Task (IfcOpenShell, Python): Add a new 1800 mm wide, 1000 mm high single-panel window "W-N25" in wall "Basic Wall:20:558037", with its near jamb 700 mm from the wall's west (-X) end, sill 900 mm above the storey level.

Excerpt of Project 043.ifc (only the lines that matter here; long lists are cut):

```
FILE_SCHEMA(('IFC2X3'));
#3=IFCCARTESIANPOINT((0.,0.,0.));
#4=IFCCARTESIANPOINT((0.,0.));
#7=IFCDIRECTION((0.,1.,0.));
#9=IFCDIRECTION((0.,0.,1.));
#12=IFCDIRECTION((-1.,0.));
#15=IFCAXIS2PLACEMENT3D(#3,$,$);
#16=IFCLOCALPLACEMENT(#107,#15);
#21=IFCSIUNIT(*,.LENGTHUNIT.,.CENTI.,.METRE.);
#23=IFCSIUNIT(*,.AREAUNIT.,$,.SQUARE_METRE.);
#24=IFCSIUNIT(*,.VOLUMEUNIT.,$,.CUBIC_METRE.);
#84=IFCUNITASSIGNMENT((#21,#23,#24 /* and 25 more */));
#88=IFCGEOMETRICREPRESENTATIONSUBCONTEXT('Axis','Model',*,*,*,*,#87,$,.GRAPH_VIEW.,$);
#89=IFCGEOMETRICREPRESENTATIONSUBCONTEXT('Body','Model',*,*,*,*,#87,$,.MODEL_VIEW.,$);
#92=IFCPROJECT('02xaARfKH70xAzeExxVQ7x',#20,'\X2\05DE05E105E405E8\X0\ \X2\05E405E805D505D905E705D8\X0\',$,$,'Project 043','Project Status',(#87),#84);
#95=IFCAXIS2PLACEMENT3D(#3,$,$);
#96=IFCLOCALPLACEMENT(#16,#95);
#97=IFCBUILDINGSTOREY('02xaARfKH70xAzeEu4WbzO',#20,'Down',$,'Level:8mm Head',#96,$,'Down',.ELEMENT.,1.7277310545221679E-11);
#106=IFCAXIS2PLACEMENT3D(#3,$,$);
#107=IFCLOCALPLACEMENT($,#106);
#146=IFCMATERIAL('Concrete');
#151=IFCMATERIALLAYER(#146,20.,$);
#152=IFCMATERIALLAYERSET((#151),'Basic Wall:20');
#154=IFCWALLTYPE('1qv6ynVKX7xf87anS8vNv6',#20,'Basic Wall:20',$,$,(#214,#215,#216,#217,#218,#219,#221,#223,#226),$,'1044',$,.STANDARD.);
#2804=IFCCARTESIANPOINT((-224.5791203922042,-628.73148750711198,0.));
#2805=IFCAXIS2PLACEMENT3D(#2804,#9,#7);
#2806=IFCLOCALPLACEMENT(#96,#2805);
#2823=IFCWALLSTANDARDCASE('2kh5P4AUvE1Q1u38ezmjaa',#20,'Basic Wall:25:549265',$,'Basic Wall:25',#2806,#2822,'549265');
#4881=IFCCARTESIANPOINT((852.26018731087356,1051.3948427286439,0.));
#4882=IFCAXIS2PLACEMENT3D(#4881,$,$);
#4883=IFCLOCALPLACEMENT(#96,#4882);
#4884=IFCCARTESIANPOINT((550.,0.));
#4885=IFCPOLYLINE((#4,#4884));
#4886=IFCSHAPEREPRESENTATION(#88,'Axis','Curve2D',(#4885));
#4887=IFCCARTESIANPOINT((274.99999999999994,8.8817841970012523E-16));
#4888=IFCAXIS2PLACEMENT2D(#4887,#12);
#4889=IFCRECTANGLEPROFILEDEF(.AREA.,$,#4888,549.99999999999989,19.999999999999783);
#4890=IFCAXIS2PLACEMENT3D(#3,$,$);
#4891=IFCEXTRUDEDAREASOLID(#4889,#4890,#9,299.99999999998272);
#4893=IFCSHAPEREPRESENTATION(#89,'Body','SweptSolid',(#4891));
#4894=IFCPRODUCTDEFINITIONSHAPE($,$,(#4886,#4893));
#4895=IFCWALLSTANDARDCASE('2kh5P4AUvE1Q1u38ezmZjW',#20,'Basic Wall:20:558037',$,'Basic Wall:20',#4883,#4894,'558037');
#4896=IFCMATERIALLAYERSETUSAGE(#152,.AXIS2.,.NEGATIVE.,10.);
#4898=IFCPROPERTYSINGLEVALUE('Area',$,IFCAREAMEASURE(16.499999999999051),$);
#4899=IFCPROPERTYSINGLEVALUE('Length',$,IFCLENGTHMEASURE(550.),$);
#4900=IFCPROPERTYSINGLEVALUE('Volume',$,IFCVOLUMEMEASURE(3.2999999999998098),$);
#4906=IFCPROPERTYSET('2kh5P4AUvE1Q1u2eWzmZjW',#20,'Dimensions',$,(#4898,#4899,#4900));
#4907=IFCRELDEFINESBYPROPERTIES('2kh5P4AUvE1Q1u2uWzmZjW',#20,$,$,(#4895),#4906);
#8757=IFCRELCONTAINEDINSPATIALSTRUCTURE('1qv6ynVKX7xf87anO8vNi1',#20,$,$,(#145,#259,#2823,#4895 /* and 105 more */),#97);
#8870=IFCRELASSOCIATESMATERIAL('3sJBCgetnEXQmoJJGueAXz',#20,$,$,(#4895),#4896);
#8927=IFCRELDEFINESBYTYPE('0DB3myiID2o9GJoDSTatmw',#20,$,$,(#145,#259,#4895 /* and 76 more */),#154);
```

```python
import numpy as np
import ifcopenshell
import ifcopenshell.api.feature
import ifcopenshell.api.geometry
import ifcopenshell.api.pset
import ifcopenshell.api.root
import ifcopenshell.api.spatial
import ifcopenshell.api.type
import ifcopenshell.geom
import ifcopenshell.util.element
import ifcopenshell.util.placement
import ifcopenshell.util.representation
import ifcopenshell.util.shape
import ifcopenshell.util.unit

model = ifcopenshell.open("Project 043.ifc")
unit_scale = ifcopenshell.util.unit.calculate_unit_scale(model)
area_scale = ifcopenshell.util.unit.calculate_unit_scale(model, "AREAUNIT")
volume_scale = ifcopenshell.util.unit.calculate_unit_scale(model, "VOLUMEUNIT")
settings = ifcopenshell.geom.settings()


def volume(element):
    """Net volume in cubic metres, openings subtracted."""
    shape = ifcopenshell.geom.create_shape(settings, element)
    return ifcopenshell.util.shape.get_volume(shape.geometry)


wall = model.by_id(4895)
storey = ifcopenshell.util.element.get_container(wall, ifc_class="IfcBuildingStorey")
context = ifcopenshell.util.representation.get_context(model, "Model", "Body", "MODEL_VIEW")
before = volume(wall)

width, height, from_end, sill = 1.8, 1, 0.7, 0.9  # metres

# The wall runs along its own X axis, and the end named is its -X end.
wall_shape = ifcopenshell.geom.create_shape(settings, wall)
x, y, z = ifcopenshell.util.shape.get_vertices(wall_shape.geometry).T
start = x.min() + from_end
face, thickness = float(y.min()), float(y.max() - y.min())
wall_matrix = ifcopenshell.util.placement.get_local_placement(wall.ObjectPlacement)
level = ifcopenshell.util.placement.get_local_placement(storey.ObjectPlacement)[2, 3]


def in_wall(x, y):
    """Placement at x, y metres in the wall's axes, at sill height."""
    matrix = wall_matrix.copy()
    matrix[:, 3] = wall_matrix @ np.array([x / unit_scale, y / unit_scale, 0.0, 1.0])
    matrix[2, 3] = level + sill / unit_scale
    return matrix


# Opening: a box that overshoots both wall faces by 50 mm.
opening = ifcopenshell.api.root.create_entity(model, ifc_class="IfcOpeningElement")
box = ifcopenshell.api.geometry.add_wall_representation(
    model, context=context, length=width, height=height, thickness=thickness + 0.1
)
ifcopenshell.api.geometry.assign_representation(model, product=opening, representation=box)
ifcopenshell.api.geometry.edit_object_placement(model, product=opening, matrix=in_wall(start, face - 0.05), is_si=False)
ifcopenshell.api.feature.add_feature(model, feature=opening, element=wall)

window = ifcopenshell.api.root.create_entity(model, ifc_class="IfcWindow", name="W-N25")
window.OverallWidth, window.OverallHeight = width / unit_scale, height / unit_scale
body = ifcopenshell.api.geometry.add_window_representation(
    model,
    context=context,
    overall_width=window.OverallWidth,
    overall_height=window.OverallHeight,
    partition_type="SINGLE_PANEL",
)
ifcopenshell.api.geometry.assign_representation(model, product=window, representation=body)
ifcopenshell.api.spatial.assign_container(model, products=[window], relating_structure=storey)
fills = ifcopenshell.api.feature.add_filling(model, opening=opening, element=window)
fills.OwnerHistory = window.OwnerHistory  # required in IFC2X3

# IFC2X3 keeps the operation on the window style.
style = ifcopenshell.api.root.create_entity(model, ifc_class="IfcWindowStyle", name="W-N25")
style.OperationType, style.ConstructionType = "SINGLE_PANEL", "NOTDEFINED"
style.ParameterTakesPrecedence = style.Sizeable = False
ifcopenshell.api.type.assign_type(model, related_objects=[window], relating_type=style)

# Centre the window in the wall's thickness.
ifcopenshell.api.geometry.edit_object_placement(model, product=window, matrix=in_wall(start, face), is_si=False)
window_shape = ifcopenshell.geom.create_shape(settings, window)
depth = ifcopenshell.util.shape.get_vertices(window_shape.geometry)[:, 1]
offset = face + thickness / 2 - (depth.min() + depth.max()) / 2
ifcopenshell.api.geometry.edit_object_placement(model, product=window, matrix=in_wall(start, offset), is_si=False)

after = volume(wall)

# Update the wall's stored quantities.
pset = model.by_id(ifcopenshell.util.element.get_pset(wall, "Dimensions", should_inherit=False)["id"])
ifcopenshell.api.pset.edit_pset(model, pset=pset, properties={
    "Area": model.create_entity("IfcAreaMeasure", after / thickness / area_scale),
    "Volume": model.create_entity("IfcVolumeMeasure", after / volume_scale),
})

print(f"wall volume {before:.3f} -> {after:.3f} m3")

model.write("Project 043-out.ifc")
```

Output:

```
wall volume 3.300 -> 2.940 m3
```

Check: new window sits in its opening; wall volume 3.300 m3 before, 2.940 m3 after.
